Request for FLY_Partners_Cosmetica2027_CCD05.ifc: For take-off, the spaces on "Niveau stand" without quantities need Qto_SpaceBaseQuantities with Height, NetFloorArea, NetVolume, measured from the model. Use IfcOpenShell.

First a look at what the model holds.

```python
import ifcopenshell
import ifcopenshell.util.element
import ifcopenshell.util.unit

model = ifcopenshell.open("FLY_Partners_Cosmetica2027_CCD05.ifc")
print(model.schema)
for unit_type in ("LENGTHUNIT", "AREAUNIT", "VOLUMEUNIT"):
    print(unit_type, ifcopenshell.util.unit.calculate_unit_scale(model, unit_type))
storey = next(s for s in model.by_type("IfcBuildingStorey") if s.Name == "Niveau stand")
spaces = [e for e in ifcopenshell.util.element.get_decomposition(storey) if e.is_a("IfcSpace")]
for e in sorted(spaces, key=lambda e: e.id()):
    print(e.id(), e.is_a(), e.Name, list(ifcopenshell.util.element.get_psets(e, qtos_only=True)), sep=" | ")
```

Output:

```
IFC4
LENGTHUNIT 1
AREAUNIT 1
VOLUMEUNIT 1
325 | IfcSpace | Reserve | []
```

```python
import ifcopenshell
import ifcopenshell.api.pset
import ifcopenshell.geom
import ifcopenshell.util.element
import ifcopenshell.util.shape
import ifcopenshell.util.unit

model = ifcopenshell.open("FLY_Partners_Cosmetica2027_CCD05.ifc")
unit_scale = ifcopenshell.util.unit.calculate_unit_scale(model)
area_scale = ifcopenshell.util.unit.calculate_unit_scale(model, "AREAUNIT")
volume_scale = ifcopenshell.util.unit.calculate_unit_scale(model, "VOLUMEUNIT")
settings = ifcopenshell.geom.settings()

storey = next(s for s in model.by_type("IfcBuildingStorey") if s.Name == "Niveau stand")
spaces = [e for e in ifcopenshell.util.element.get_decomposition(storey) if e.is_a("IfcSpace")]

for e in sorted(spaces, key=lambda e: e.id()):
    if ifcopenshell.util.element.get_psets(e, qtos_only=True, should_inherit=False):
        continue
    # Geometry comes back in metres, in the element's own axes.
    shape = ifcopenshell.geom.create_shape(settings, e)
    values = {
        "Height": ifcopenshell.util.shape.get_z(shape.geometry) / unit_scale,
        "NetFloorArea": ifcopenshell.util.shape.get_footprint_area(shape.geometry) / area_scale,
        "NetVolume": ifcopenshell.util.shape.get_volume(shape.geometry) / volume_scale,
    }
    qto = ifcopenshell.api.pset.add_qto(model, product=e, name="Qto_SpaceBaseQuantities")
    ifcopenshell.api.pset.edit_qto(model, qto=qto, properties=values)
    print(e.id(), {k: round(v, 3) for k, v in values.items()})

model.write("FLY_Partners_Cosmetica2027_CCD05_updated.ifc")
```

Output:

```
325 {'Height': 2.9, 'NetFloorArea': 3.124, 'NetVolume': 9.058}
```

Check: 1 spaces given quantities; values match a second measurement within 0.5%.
